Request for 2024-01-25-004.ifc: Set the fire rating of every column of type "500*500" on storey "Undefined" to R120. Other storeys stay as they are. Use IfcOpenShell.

First a look at what the model holds.

```python
import ifcopenshell
import ifcopenshell.util.element

model = ifcopenshell.open("2024-01-25-004.ifc")
print(model.schema)
storey = next(s for s in model.by_type("IfcBuildingStorey") if s.Name == "Undefined")
columns = [e for e in ifcopenshell.util.element.get_decomposition(storey) if e.is_a("IfcColumn")]
seen = {}
for e in columns:
    element_type = ifcopenshell.util.element.get_type(e)
    key = (element_type.Name if element_type != e and element_type else None, ifcopenshell.util.element.get_pset(e, "Pset_ColumnCommon", "FireRating"))
    seen[key] = seen.get(key, 0) + 1
for (name, value), count in sorted(seen.items(), key=str):
    print(count, "x", name, "|", value)
```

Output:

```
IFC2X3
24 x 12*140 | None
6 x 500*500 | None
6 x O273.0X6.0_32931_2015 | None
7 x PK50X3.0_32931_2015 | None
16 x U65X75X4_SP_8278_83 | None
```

```python
import ifcopenshell
import ifcopenshell.api.pset
import ifcopenshell.util.element

model = ifcopenshell.open("2024-01-25-004.ifc")

storey = next(s for s in model.by_type("IfcBuildingStorey") if s.Name == "Undefined")
columns = [e for e in ifcopenshell.util.element.get_decomposition(storey) if e.is_a("IfcColumn")]

count = 0
for e in columns:
    element_type = ifcopenshell.util.element.get_type(e)
    if element_type in (None, e) or element_type.Name != "500*500":
        continue
    found = ifcopenshell.util.element.get_pset(e, "Pset_ColumnCommon", should_inherit=False)
    if found:
        pset = model.by_id(found["id"])
        if len(ifcopenshell.util.element.get_elements_by_pset(pset)) > 1:
            pset = ifcopenshell.api.pset.unshare_pset(model, products=[e], pset=pset)[0]
    else:
        pset = ifcopenshell.api.pset.add_pset(model, product=e, name="Pset_ColumnCommon")
    ifcopenshell.api.pset.edit_pset(model, pset=pset, properties={"FireRating": "R120"})
    count += 1

print(count, "columns updated")

model.write("2024-01-25-004_rev.ifc")
```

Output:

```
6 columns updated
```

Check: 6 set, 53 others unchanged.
